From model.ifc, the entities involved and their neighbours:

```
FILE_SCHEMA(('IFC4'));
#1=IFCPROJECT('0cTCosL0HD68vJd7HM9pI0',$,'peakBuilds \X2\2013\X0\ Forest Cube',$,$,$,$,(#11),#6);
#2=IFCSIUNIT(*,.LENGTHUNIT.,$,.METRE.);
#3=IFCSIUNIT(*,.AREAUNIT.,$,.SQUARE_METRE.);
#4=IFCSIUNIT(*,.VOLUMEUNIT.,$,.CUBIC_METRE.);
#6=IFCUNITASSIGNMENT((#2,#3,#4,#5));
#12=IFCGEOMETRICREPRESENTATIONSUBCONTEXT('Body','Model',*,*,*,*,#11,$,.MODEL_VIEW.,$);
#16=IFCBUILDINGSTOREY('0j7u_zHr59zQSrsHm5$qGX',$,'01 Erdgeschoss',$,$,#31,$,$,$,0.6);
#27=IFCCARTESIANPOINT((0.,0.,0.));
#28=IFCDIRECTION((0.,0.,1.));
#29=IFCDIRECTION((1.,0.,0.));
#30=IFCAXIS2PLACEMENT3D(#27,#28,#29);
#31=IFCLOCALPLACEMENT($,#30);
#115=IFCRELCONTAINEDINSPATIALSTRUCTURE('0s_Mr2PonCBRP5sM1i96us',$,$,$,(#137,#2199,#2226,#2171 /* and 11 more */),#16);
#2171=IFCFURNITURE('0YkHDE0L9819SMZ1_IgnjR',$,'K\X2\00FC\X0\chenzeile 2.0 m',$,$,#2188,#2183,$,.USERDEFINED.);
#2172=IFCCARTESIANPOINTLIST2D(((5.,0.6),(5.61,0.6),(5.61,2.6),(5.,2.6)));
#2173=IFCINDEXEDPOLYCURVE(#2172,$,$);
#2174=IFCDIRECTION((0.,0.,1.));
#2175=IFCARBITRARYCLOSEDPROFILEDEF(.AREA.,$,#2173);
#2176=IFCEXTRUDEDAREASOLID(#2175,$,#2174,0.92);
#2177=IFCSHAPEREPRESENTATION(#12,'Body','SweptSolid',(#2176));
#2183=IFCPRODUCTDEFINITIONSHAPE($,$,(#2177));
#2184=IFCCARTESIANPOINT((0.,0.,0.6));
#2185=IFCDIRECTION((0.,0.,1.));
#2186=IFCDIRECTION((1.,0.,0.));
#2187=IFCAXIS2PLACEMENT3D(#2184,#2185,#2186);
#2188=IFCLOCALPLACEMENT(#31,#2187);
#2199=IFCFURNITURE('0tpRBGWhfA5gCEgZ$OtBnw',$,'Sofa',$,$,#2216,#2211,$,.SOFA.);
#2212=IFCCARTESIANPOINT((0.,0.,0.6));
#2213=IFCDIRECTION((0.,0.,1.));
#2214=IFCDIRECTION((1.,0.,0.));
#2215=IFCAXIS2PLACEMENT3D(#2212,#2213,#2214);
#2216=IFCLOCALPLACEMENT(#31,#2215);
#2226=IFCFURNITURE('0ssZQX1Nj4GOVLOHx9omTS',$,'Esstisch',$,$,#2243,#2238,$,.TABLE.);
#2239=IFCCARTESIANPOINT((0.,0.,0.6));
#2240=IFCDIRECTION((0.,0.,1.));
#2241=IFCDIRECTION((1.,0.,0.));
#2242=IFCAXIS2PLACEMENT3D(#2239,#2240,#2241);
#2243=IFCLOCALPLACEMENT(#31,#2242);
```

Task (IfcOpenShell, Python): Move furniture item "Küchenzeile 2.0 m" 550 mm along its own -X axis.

```python
import ifcopenshell
import ifcopenshell.api.geometry
import ifcopenshell.util.placement

model = ifcopenshell.open("model.ifc")

item = model.by_guid("0YkHDE0L9819SMZ1_IgnjR")
matrix = ifcopenshell.util.placement.get_local_placement(item.ObjectPlacement)
matrix[:3, 3] -= matrix[:3, 0] * 0.55
ifcopenshell.api.geometry.edit_object_placement(model, product=item, matrix=matrix, is_si=False)

print(ifcopenshell.util.placement.get_local_placement(item.ObjectPlacement).round(3) + 0.0)

model.write("model_rev.ifc")
```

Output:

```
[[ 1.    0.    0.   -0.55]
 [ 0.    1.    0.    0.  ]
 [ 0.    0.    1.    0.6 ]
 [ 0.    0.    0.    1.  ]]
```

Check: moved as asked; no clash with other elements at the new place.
